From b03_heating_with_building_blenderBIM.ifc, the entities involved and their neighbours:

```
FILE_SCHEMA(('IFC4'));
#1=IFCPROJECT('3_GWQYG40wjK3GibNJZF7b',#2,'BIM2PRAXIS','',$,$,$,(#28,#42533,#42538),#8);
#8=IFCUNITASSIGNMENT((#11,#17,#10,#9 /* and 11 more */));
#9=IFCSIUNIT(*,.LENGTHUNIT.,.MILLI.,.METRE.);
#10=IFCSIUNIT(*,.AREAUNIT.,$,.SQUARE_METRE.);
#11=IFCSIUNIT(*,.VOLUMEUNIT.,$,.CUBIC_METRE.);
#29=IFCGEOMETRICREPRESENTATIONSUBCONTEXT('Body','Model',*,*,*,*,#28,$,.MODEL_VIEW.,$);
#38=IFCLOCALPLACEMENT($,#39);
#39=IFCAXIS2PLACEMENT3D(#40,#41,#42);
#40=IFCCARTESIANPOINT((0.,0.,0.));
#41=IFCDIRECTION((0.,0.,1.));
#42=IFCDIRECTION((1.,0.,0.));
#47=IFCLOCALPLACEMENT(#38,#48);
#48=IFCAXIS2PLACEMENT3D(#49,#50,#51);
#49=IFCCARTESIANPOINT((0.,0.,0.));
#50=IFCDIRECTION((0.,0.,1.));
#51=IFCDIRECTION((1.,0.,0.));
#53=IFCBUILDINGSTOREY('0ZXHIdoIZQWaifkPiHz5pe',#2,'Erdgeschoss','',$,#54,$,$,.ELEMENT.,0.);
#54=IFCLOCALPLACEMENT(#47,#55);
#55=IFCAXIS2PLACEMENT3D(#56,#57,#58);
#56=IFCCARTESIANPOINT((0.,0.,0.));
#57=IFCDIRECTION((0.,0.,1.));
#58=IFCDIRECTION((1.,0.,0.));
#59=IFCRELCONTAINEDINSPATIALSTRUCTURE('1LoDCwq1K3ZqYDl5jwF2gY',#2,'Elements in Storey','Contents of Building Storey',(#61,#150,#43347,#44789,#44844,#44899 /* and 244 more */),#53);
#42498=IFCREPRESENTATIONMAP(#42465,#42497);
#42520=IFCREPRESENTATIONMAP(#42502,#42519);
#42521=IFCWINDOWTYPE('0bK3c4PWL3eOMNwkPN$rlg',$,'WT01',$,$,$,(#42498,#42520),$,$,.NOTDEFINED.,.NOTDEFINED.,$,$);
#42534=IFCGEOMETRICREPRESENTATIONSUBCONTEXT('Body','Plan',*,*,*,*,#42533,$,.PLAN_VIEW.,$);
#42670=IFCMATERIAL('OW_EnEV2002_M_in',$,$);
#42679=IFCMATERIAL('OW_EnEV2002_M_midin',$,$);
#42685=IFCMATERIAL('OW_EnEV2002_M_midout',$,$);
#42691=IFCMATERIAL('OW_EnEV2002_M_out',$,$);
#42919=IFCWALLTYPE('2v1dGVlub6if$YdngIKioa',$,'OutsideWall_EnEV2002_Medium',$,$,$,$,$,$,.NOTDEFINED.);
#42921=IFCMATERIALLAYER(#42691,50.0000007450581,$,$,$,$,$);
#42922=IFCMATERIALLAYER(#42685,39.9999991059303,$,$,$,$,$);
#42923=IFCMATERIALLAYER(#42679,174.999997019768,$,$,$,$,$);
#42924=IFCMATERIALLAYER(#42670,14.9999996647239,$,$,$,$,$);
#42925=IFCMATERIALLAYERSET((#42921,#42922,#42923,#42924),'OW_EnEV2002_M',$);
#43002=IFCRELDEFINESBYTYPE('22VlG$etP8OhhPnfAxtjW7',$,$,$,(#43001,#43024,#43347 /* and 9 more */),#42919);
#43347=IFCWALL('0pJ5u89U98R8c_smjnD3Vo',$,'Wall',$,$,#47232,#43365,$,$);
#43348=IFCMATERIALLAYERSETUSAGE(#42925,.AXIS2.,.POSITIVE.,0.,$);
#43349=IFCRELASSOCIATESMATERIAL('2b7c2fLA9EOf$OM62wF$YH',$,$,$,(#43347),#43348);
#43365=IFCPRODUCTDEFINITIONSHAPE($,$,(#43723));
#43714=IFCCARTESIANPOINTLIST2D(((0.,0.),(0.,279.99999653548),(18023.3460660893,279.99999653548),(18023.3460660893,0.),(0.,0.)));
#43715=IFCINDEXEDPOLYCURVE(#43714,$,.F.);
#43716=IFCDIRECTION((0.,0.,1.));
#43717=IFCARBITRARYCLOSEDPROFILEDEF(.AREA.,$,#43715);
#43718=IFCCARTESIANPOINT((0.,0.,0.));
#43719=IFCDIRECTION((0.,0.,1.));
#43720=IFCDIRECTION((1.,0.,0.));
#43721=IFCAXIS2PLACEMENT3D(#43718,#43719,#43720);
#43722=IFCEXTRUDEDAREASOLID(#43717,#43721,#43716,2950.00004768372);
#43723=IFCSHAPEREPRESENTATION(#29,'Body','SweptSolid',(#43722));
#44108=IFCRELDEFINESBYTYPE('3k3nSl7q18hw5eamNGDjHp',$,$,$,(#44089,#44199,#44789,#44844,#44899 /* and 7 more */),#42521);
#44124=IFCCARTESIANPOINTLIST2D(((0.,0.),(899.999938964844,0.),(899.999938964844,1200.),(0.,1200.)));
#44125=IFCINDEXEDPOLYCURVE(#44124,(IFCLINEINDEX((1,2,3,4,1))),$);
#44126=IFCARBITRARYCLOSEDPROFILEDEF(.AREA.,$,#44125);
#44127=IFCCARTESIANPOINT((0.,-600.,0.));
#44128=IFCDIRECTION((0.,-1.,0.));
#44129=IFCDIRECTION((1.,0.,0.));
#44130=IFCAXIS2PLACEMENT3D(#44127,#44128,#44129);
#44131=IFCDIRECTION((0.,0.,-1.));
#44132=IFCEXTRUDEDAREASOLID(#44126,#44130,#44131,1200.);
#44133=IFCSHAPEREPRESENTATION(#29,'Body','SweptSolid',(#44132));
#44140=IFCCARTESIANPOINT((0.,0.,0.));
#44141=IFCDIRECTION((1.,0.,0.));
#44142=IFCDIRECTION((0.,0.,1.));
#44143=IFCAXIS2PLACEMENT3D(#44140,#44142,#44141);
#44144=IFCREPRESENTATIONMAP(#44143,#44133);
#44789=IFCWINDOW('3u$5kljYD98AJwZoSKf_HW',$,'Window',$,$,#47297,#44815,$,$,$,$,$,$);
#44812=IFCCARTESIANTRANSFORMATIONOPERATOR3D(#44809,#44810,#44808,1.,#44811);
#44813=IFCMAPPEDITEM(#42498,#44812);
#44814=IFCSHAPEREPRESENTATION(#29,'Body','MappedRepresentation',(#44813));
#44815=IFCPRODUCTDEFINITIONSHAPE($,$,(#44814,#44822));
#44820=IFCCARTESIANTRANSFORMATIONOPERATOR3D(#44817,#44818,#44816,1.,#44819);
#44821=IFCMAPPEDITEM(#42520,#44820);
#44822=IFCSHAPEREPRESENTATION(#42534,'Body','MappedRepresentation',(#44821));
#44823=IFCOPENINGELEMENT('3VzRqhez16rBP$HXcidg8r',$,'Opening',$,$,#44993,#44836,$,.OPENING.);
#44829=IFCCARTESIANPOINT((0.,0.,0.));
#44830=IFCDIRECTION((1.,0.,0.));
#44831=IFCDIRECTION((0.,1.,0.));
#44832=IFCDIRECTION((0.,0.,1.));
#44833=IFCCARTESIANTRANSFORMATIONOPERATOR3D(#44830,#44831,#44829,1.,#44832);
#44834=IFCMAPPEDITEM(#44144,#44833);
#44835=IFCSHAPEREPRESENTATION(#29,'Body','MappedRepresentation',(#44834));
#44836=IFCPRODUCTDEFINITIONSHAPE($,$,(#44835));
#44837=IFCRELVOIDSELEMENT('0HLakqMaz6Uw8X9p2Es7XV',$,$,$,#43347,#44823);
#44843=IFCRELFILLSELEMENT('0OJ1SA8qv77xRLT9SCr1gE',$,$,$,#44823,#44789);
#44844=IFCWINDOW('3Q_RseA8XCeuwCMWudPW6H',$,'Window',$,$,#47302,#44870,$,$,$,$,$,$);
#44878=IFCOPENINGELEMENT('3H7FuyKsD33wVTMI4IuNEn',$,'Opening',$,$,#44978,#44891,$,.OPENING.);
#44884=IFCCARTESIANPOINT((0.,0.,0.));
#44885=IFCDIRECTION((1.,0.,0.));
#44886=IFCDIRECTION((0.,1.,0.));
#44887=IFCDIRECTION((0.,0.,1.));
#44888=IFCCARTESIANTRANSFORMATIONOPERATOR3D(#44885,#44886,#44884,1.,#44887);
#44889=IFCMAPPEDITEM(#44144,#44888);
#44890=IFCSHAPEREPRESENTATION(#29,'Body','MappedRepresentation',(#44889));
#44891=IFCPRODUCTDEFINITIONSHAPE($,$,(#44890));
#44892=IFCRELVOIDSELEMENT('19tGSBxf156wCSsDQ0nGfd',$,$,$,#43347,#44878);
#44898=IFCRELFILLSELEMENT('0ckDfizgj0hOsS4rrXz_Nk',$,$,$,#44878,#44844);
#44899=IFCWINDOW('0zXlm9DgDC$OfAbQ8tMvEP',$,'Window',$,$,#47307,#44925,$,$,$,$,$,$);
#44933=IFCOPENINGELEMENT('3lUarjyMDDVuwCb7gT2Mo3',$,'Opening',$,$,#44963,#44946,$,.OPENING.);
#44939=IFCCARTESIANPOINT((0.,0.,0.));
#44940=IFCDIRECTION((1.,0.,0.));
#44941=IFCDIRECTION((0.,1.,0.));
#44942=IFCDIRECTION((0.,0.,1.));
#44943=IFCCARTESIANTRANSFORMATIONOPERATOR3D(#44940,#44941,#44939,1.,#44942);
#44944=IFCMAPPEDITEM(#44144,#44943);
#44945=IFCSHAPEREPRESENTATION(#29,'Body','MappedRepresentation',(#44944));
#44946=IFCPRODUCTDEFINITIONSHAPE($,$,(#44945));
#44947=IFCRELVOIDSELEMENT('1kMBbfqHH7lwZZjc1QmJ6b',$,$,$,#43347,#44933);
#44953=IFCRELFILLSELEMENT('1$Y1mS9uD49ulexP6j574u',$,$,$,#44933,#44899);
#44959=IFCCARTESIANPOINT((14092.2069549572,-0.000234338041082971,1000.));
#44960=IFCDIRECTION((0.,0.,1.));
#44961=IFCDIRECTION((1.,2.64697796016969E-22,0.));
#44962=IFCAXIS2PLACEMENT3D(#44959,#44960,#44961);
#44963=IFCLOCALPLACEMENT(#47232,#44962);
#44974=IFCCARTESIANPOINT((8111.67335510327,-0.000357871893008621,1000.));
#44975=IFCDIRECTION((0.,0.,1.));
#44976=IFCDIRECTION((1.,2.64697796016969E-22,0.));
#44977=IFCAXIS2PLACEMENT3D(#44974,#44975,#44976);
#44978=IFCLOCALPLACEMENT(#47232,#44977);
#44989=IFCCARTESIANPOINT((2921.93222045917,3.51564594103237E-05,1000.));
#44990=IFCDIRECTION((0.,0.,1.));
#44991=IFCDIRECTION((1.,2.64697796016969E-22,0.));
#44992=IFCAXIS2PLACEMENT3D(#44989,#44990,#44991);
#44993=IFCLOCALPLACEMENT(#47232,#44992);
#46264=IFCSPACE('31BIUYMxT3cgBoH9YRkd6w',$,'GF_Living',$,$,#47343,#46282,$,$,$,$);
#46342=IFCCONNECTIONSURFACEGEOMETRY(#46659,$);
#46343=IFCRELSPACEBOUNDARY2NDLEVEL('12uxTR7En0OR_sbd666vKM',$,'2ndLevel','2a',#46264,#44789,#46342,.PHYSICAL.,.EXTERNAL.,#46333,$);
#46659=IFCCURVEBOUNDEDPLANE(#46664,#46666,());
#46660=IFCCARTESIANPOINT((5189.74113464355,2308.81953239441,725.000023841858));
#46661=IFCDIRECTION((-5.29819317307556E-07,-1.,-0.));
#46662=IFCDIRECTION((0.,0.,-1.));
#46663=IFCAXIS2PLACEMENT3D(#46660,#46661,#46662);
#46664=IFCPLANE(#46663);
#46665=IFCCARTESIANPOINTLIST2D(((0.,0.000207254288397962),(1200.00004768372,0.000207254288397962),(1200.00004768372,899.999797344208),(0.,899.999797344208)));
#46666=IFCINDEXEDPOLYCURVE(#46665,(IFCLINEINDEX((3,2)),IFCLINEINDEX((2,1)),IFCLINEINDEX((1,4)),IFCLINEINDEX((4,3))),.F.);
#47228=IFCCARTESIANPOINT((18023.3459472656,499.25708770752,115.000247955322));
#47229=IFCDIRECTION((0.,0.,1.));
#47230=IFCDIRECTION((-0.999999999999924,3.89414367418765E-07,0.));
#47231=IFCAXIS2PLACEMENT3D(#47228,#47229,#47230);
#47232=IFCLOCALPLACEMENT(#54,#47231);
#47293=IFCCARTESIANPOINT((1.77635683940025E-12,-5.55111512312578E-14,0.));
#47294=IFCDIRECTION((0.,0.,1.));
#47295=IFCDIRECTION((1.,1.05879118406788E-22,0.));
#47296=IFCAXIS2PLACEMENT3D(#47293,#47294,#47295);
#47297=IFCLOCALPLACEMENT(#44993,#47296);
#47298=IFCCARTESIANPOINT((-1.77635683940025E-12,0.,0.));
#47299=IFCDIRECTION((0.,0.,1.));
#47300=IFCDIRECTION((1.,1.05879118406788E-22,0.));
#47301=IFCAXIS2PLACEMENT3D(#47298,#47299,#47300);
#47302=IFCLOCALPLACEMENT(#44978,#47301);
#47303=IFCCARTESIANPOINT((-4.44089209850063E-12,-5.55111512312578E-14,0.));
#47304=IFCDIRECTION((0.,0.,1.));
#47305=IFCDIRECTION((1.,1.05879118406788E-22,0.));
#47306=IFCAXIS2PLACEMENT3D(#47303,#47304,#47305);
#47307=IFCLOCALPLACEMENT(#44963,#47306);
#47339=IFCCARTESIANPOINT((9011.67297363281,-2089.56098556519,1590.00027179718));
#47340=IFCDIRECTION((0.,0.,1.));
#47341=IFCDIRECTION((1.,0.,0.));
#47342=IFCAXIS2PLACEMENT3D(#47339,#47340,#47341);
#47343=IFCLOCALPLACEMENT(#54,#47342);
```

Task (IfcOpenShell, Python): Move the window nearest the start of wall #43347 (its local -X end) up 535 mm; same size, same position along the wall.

```python
import numpy as np
import ifcopenshell
import ifcopenshell.api.geometry
import ifcopenshell.util.placement
import ifcopenshell.util.unit

model = ifcopenshell.open("b03_heating_with_building_blenderBIM.ifc")
unit_scale = ifcopenshell.util.unit.calculate_unit_scale(model)

window = model.by_guid("3u$5kljYD98AJwZoSKf_HW")
opening = window.FillsVoids[0].RelatingOpeningElement
dz = 0.535 / unit_scale

shift = np.array([0.0, 0.0, dz])
# The window is placed relative to its opening, so it follows when the opening moves.
matrix = ifcopenshell.util.placement.get_local_placement(opening.ObjectPlacement)
matrix[:3, 3] += shift
ifcopenshell.api.geometry.edit_object_placement(
    model, product=opening, matrix=matrix, is_si=False, should_transform_children=True
)

# Space boundary surfaces are stored in each space's coordinates; move them too.
for rel in window.ProvidesBoundaries:
    if not rel.ConnectionGeometry:
        continue
    surface = rel.ConnectionGeometry.SurfaceOnRelatingElement.BasisSurface
    space_matrix = ifcopenshell.util.placement.get_local_placement(rel.RelatingSpace.ObjectPlacement)
    point = np.array(surface.Position.Location.Coordinates) + space_matrix[:3, :3].T @ shift
    surface.Position = model.createIfcAxis2Placement3D(
        model.createIfcCartesianPoint(point.tolist()), surface.Position.Axis, surface.Position.RefDirection
    )

print(f"moved by {dz * unit_scale:+.3f} m")

model.write("b03_heating_with_building_blenderBIM_rev.ifc")
```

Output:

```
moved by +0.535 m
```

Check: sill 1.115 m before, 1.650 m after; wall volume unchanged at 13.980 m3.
